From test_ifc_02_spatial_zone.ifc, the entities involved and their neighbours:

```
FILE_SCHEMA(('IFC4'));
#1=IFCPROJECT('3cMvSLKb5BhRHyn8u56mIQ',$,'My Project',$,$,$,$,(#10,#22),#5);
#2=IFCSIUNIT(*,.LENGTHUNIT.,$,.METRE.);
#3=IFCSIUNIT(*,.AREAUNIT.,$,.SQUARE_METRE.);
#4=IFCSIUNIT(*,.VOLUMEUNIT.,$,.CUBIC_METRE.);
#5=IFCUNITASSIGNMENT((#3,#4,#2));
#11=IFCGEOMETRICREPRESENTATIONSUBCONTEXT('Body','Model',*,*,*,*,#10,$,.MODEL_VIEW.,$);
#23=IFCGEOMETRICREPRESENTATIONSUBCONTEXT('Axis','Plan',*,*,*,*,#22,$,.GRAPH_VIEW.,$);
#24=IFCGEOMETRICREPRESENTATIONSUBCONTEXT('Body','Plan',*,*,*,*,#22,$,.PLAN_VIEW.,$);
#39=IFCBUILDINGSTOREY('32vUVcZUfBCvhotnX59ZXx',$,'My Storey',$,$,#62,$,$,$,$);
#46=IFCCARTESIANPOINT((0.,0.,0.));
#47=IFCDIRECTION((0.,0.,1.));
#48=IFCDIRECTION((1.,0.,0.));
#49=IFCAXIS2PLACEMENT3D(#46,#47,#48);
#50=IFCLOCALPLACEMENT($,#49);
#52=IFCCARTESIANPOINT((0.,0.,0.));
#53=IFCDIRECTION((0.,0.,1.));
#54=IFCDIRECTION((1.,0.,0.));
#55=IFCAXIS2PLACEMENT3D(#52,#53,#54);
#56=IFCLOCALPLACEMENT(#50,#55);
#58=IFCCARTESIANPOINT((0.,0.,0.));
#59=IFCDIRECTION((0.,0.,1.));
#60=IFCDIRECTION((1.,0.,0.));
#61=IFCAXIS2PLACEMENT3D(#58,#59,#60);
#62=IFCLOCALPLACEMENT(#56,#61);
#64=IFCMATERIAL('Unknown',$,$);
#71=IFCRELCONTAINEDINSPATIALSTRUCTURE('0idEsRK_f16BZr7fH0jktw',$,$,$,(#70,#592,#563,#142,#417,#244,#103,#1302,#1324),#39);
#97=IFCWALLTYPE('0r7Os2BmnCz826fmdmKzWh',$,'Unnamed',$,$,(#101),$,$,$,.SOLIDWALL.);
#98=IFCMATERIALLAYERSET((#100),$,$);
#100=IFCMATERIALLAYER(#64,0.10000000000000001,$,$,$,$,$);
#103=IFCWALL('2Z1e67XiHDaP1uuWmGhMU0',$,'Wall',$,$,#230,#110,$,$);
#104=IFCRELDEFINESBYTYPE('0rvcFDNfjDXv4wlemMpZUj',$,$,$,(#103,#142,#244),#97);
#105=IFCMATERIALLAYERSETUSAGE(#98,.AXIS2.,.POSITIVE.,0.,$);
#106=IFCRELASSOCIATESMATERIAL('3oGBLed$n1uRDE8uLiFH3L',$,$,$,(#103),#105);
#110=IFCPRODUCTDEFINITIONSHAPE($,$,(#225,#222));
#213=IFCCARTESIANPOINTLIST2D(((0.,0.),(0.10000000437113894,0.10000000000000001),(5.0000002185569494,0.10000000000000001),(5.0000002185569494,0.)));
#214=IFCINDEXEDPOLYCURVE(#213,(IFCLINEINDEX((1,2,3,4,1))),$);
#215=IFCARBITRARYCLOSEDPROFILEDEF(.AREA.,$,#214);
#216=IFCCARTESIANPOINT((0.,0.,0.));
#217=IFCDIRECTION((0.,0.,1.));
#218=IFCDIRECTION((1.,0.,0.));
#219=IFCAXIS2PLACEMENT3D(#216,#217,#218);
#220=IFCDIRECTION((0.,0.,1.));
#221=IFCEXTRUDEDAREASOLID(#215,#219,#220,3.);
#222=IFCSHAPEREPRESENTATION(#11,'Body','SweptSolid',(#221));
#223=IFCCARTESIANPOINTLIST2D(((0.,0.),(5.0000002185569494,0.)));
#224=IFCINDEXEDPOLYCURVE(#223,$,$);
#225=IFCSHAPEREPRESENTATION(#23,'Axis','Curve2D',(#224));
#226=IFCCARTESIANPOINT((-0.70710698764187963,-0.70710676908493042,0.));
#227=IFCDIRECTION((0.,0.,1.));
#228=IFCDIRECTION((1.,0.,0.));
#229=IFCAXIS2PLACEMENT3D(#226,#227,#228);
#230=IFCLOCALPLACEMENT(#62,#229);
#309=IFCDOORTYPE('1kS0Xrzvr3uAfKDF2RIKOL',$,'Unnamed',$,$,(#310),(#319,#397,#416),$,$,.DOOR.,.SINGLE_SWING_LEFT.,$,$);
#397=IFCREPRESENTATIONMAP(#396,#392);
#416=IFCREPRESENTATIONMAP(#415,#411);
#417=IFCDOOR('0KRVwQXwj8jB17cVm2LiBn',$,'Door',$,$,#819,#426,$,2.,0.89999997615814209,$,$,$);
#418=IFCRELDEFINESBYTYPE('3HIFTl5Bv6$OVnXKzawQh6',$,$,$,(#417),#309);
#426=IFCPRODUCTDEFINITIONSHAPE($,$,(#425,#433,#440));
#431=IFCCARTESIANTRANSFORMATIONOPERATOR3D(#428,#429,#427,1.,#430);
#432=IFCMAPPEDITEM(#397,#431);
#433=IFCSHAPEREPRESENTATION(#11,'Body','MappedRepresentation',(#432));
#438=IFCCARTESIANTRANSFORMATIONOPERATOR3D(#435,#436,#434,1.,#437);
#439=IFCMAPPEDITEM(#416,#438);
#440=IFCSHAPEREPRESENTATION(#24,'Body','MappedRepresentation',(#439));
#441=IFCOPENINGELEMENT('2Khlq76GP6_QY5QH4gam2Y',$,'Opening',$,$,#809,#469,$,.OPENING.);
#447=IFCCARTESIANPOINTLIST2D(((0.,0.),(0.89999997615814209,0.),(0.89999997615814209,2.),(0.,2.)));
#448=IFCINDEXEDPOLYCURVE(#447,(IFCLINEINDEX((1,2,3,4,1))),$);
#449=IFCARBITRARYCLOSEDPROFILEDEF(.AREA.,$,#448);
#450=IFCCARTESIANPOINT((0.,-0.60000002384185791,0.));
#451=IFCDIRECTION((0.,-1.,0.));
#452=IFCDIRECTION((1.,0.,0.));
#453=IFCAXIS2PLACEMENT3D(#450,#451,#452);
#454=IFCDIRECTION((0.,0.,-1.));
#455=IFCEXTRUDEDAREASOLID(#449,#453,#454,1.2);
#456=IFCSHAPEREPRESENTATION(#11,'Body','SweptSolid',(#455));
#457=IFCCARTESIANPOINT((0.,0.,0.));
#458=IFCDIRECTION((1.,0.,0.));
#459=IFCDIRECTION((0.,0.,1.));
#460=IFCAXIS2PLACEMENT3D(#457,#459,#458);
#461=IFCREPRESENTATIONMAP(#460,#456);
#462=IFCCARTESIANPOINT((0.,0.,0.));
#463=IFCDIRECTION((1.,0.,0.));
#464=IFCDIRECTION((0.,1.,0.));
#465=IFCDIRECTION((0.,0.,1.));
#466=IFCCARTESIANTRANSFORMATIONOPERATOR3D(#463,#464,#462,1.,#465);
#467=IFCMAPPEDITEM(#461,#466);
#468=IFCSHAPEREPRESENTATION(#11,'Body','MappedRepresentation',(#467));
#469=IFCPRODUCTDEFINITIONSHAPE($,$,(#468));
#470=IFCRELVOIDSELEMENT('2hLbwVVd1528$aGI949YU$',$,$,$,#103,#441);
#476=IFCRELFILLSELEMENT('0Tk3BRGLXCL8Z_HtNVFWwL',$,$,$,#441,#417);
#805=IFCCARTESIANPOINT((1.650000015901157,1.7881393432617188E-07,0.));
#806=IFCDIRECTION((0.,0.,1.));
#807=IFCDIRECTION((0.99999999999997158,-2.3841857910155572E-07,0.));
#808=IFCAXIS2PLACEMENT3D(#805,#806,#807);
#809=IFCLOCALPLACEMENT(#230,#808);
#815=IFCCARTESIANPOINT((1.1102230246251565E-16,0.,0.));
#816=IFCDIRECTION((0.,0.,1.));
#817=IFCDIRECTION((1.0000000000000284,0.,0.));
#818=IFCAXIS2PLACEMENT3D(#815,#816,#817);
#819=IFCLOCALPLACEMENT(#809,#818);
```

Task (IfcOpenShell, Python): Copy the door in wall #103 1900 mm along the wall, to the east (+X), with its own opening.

```python
import ifcopenshell
import ifcopenshell.api.feature
import ifcopenshell.api.geometry
import ifcopenshell.api.root
import ifcopenshell.geom
import ifcopenshell.util.element
import ifcopenshell.util.placement
import ifcopenshell.util.shape
import ifcopenshell.util.unit

model = ifcopenshell.open("test_ifc_02_spatial_zone.ifc")
unit_scale = ifcopenshell.util.unit.calculate_unit_scale(model)
settings = ifcopenshell.geom.settings()


def volume(element):
    """Net volume in cubic metres, openings subtracted."""
    shape = ifcopenshell.geom.create_shape(settings, element)
    return ifcopenshell.util.shape.get_volume(shape.geometry)


door = model.by_guid("0KRVwQXwj8jB17cVm2LiBn")
opening = door.FillsVoids[0].RelatingOpeningElement
wall = opening.VoidsElements[0].RelatingBuildingElement
before = volume(wall)
shift = ifcopenshell.util.placement.get_local_placement(wall.ObjectPlacement)[:3, 0] * 1.9 / unit_scale

# copy_class copies the void relationship, type, container and properties, but no geometry.
new_opening = ifcopenshell.api.root.copy_class(model, product=opening)
new_opening.Representation = ifcopenshell.util.element.copy_deep(
    model, opening.Representation, exclude=["IfcGeometricRepresentationContext", "IfcRepresentationMap"]
)
new_door = ifcopenshell.api.root.copy_class(model, product=door)
new_door.Representation = ifcopenshell.util.element.copy_deep(
    model, door.Representation, exclude=["IfcGeometricRepresentationContext", "IfcRepresentationMap"]
)
ifcopenshell.api.feature.add_filling(model, opening=new_opening, element=new_door)

for old, new in ((opening, new_opening), (door, new_door)):
    matrix = ifcopenshell.util.placement.get_local_placement(old.ObjectPlacement)
    matrix[:3, 3] += shift
    ifcopenshell.api.geometry.edit_object_placement(model, product=new, matrix=matrix, is_si=False)

after = volume(wall)

print(f"wall volume {before:.3f} -> {after:.3f} m3")

model.write("test_ifc_02_spatial_zone-out.ifc")
```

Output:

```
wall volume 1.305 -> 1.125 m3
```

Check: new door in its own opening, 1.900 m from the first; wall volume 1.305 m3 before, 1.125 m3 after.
